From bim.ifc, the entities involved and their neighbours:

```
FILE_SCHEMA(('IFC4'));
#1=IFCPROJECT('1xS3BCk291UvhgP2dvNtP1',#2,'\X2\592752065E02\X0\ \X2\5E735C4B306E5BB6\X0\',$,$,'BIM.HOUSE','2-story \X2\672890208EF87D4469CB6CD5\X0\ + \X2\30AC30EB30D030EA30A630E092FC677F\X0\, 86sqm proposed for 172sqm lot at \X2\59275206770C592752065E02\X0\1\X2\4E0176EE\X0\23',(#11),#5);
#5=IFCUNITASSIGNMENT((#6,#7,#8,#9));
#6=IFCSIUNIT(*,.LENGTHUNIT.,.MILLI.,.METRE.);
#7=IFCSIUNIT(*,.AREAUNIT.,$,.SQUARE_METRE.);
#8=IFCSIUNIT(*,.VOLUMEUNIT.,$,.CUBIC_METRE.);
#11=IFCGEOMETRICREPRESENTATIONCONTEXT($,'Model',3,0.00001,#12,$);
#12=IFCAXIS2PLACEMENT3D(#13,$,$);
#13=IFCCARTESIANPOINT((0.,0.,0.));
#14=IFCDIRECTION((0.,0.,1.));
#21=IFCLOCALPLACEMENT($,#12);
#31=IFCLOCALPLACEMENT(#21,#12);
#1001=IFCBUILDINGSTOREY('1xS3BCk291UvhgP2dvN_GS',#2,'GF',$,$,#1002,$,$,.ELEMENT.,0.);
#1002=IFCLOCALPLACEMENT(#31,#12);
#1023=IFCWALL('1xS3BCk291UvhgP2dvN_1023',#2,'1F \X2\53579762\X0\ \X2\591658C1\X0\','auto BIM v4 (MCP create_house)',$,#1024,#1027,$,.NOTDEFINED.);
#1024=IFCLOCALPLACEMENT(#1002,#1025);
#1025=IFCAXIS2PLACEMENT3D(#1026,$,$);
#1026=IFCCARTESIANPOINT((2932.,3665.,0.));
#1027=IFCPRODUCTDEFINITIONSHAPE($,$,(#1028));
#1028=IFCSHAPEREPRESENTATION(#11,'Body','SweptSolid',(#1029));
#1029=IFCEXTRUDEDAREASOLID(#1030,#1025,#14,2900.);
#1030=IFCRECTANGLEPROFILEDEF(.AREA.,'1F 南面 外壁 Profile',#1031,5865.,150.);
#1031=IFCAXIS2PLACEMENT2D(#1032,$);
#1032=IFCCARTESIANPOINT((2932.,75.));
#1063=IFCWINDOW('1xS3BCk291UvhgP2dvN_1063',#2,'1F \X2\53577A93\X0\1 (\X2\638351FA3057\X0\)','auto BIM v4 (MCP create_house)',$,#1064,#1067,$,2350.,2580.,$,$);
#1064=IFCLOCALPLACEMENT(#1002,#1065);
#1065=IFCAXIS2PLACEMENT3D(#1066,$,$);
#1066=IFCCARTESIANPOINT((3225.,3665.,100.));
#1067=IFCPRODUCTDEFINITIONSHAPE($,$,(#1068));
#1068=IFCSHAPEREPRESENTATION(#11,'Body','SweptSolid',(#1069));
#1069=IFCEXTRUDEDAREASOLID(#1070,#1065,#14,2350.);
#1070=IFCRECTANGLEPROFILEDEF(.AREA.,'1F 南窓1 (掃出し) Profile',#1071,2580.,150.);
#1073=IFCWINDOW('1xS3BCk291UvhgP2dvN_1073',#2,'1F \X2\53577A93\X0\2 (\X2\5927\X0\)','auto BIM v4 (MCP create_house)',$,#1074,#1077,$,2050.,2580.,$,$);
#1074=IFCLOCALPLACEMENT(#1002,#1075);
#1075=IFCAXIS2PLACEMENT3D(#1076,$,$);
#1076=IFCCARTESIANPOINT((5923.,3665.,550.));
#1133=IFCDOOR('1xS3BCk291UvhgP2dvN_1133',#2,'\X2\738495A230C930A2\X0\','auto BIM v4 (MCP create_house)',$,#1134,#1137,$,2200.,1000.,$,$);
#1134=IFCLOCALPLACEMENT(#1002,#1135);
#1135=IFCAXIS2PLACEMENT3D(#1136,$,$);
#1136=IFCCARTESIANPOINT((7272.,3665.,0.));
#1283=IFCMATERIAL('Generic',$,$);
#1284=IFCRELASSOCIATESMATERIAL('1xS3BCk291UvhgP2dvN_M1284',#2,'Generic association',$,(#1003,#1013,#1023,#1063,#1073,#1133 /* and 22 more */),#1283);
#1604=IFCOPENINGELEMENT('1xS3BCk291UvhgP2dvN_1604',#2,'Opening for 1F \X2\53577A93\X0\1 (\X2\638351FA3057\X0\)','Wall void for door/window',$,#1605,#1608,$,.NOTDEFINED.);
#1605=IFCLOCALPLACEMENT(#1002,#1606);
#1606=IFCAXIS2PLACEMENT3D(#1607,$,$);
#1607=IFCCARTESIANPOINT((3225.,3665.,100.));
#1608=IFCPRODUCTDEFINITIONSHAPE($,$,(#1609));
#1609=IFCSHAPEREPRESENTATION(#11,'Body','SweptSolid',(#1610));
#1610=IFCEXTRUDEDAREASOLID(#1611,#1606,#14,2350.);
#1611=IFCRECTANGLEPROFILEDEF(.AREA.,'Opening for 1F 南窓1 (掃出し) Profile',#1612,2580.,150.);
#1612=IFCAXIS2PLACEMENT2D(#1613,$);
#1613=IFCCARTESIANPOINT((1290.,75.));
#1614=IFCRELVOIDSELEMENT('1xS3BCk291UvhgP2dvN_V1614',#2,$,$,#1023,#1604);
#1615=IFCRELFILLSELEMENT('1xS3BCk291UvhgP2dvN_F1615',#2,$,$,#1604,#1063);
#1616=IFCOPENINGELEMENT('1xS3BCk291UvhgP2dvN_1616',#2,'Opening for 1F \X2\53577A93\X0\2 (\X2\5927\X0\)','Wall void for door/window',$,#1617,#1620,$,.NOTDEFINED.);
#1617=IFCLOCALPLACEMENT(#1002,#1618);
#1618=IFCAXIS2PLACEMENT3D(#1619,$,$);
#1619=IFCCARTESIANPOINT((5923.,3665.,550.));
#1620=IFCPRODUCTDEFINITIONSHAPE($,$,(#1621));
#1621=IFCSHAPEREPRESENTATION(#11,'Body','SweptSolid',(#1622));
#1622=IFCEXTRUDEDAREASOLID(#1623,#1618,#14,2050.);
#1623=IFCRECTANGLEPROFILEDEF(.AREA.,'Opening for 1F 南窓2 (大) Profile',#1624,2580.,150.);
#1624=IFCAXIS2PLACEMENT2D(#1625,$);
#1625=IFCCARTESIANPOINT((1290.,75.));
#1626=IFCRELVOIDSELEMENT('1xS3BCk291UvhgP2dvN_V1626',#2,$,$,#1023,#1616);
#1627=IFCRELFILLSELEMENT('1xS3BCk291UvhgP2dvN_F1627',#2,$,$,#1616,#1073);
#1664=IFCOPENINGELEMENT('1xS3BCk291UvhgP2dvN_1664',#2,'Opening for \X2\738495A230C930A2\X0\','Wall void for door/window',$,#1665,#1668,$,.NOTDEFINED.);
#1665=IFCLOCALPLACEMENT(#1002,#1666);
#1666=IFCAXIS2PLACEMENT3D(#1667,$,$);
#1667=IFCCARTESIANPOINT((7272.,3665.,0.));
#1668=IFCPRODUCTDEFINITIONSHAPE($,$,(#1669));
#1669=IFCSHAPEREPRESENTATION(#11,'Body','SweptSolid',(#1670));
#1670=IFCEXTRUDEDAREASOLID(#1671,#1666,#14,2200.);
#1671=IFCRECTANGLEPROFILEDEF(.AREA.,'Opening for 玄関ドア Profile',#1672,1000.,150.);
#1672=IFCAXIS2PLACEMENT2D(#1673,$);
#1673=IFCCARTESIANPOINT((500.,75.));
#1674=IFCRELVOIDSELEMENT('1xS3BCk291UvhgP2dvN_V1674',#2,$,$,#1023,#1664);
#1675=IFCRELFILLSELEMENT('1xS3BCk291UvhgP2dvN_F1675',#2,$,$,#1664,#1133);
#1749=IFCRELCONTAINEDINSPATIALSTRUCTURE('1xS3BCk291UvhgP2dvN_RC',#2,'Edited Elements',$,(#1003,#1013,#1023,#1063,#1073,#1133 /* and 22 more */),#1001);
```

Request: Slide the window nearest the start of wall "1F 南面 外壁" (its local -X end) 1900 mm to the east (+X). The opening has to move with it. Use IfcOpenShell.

```python
import ifcopenshell
import ifcopenshell.api.geometry
import ifcopenshell.util.placement
import ifcopenshell.util.unit

model = ifcopenshell.open("bim.ifc")
unit_scale = ifcopenshell.util.unit.calculate_unit_scale(model)

window = model.by_guid("1xS3BCk291UvhgP2dvN_1063")
opening = window.FillsVoids[0].RelatingOpeningElement
wall = opening.VoidsElements[0].RelatingBuildingElement

wall_matrix = ifcopenshell.util.placement.get_local_placement(wall.ObjectPlacement)
shift = wall_matrix[:3, 0] * 1.9 / unit_scale
before = ifcopenshell.util.placement.get_local_placement(window.ObjectPlacement)[:3, 3].copy()

# The window is not placed relative to its opening, so move both.
for product in (opening, window):
    matrix = ifcopenshell.util.placement.get_local_placement(product.ObjectPlacement)
    matrix[:3, 3] += shift
    ifcopenshell.api.geometry.edit_object_placement(model, product=product, matrix=matrix, is_si=False)

after = ifcopenshell.util.placement.get_local_placement(window.ObjectPlacement)[:3, 3]
print("window moved by", (after - before).round(3) + 0.0)

model.write("bim_v2.ifc")
```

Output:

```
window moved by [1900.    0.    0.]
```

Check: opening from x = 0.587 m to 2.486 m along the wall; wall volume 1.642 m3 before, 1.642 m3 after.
